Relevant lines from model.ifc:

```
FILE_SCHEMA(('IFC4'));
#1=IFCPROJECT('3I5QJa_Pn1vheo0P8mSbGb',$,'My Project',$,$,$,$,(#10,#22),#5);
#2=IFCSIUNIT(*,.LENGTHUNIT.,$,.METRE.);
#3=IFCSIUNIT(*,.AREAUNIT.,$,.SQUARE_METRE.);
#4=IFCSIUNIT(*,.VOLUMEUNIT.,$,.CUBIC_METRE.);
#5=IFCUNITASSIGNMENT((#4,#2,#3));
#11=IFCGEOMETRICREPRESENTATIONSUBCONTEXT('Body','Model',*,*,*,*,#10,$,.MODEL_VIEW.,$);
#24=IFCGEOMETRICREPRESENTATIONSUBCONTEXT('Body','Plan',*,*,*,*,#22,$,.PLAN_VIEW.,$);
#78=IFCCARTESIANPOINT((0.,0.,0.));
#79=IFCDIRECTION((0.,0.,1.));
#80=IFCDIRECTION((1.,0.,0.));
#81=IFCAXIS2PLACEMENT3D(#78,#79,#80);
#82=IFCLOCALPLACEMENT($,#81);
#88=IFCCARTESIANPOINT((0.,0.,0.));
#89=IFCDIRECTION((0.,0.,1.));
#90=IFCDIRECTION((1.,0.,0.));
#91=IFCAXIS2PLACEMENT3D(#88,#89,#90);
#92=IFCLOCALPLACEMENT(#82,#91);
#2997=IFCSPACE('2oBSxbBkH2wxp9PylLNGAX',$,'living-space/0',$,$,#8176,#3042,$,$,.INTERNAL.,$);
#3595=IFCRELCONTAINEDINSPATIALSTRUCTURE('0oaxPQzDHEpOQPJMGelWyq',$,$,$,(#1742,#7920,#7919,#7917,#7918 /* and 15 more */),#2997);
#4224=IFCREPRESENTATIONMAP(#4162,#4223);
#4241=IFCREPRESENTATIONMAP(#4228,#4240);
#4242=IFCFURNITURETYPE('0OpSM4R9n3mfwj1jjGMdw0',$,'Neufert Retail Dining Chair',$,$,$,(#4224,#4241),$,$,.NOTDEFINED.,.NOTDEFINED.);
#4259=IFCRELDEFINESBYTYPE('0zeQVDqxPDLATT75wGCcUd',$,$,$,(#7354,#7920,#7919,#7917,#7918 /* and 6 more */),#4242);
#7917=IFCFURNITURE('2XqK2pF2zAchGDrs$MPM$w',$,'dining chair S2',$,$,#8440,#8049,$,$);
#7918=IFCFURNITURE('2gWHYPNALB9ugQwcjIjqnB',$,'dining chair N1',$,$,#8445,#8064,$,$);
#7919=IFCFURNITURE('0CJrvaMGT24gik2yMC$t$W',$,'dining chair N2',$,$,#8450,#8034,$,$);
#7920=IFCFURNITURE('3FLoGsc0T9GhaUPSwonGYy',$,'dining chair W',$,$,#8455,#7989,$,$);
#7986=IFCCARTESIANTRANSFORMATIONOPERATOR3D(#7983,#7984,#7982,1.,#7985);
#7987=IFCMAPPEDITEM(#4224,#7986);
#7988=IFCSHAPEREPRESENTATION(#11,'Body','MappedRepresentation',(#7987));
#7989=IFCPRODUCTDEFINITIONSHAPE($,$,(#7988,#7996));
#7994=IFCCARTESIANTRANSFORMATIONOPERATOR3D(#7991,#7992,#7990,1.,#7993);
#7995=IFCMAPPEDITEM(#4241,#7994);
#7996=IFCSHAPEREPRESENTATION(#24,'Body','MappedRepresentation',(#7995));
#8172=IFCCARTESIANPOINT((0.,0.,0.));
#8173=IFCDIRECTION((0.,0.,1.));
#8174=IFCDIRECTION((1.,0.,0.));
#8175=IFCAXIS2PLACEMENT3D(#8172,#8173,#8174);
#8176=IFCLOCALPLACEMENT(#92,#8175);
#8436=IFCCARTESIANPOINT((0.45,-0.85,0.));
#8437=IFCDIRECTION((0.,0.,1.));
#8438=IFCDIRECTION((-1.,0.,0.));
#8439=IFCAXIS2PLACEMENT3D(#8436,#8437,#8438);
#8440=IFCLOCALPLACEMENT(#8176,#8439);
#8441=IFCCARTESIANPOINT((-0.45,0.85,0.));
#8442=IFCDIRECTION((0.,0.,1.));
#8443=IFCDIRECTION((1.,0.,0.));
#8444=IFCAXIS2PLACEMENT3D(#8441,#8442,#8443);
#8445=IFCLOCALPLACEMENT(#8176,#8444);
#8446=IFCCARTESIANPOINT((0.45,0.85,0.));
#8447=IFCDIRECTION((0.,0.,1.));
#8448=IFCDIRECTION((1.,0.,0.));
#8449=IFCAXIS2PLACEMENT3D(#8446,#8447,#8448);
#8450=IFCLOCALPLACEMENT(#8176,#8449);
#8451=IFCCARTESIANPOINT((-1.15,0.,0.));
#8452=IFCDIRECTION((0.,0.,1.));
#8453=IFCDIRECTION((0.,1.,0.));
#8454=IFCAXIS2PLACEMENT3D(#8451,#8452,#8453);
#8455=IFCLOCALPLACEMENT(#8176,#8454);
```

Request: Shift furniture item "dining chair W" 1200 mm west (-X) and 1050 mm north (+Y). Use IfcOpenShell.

```python
import ifcopenshell
import ifcopenshell.api.geometry
import ifcopenshell.util.placement

model = ifcopenshell.open("model.ifc")

item = model.by_guid("3FLoGsc0T9GhaUPSwonGYy")
matrix = ifcopenshell.util.placement.get_local_placement(item.ObjectPlacement)
matrix[0, 3] -= 1.2
matrix[1, 3] += 1.05
ifcopenshell.api.geometry.edit_object_placement(model, product=item, matrix=matrix, is_si=False)

print(ifcopenshell.util.placement.get_local_placement(item.ObjectPlacement).round(3) + 0.0)

model.write("model-out.ifc")
```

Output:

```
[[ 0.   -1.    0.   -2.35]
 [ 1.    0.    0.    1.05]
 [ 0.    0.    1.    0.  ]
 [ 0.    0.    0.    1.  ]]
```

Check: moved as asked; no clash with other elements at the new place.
